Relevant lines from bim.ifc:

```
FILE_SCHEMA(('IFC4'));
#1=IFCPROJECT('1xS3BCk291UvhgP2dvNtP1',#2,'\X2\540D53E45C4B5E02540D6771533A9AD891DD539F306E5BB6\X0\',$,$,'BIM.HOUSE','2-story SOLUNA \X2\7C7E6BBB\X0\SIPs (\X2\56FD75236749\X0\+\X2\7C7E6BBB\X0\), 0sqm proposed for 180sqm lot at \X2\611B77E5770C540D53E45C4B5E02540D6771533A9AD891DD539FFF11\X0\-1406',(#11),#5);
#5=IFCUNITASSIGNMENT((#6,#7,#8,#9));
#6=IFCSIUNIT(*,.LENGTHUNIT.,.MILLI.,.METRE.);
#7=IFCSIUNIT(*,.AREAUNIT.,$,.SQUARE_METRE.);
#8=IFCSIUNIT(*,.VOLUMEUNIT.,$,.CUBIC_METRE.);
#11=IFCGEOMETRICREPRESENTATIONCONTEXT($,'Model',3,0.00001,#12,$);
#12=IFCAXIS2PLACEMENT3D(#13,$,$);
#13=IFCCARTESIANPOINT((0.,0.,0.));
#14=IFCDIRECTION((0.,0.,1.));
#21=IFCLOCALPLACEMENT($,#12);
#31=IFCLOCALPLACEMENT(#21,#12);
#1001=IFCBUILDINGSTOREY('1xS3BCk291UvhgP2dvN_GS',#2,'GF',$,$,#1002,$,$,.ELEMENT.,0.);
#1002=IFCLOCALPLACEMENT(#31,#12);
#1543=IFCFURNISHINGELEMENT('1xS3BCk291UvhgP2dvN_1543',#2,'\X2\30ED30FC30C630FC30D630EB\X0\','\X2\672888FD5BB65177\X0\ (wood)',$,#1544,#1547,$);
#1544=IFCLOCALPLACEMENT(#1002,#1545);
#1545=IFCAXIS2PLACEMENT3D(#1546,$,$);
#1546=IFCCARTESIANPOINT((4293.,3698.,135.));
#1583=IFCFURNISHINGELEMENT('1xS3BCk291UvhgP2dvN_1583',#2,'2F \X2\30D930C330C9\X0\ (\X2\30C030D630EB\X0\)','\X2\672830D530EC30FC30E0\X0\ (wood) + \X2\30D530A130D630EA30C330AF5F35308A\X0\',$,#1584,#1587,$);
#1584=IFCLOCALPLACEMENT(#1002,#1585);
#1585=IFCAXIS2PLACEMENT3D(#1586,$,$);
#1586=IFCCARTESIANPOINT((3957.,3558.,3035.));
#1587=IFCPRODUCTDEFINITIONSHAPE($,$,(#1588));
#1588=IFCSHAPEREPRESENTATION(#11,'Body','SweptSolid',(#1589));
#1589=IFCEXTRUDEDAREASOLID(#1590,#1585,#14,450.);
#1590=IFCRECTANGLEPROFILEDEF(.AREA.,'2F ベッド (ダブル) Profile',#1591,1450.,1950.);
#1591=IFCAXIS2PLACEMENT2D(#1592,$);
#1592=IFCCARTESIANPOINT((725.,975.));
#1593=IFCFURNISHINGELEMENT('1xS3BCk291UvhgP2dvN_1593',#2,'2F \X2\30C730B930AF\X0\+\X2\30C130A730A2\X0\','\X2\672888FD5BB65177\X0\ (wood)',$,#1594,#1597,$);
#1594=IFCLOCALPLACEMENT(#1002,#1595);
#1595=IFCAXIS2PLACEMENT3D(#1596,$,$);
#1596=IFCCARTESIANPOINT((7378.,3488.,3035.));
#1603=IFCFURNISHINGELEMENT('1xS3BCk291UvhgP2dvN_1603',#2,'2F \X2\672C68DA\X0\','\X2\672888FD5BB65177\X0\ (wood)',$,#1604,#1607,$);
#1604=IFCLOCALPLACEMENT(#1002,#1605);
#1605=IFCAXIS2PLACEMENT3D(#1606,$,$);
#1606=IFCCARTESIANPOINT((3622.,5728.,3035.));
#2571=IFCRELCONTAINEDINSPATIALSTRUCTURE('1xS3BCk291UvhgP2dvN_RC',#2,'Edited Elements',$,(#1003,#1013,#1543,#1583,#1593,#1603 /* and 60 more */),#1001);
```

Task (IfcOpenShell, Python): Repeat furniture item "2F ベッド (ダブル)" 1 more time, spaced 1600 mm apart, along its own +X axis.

```python
import ifcopenshell
import ifcopenshell.api.geometry
import ifcopenshell.api.root
import ifcopenshell.util.element
import ifcopenshell.util.placement

model = ifcopenshell.open("bim.ifc")


def reuse_history(source, copy):
    """copy_class also copies each property set's owner history, people and application; keep the originals."""
    for rel in copy.IsDefinedBy:
        if rel.is_a("IfcRelDefinesByProperties") and (history := rel.RelatingPropertyDefinition.OwnerHistory):
            rel.RelatingPropertyDefinition.OwnerHistory = source.OwnerHistory
            ifcopenshell.util.element.remove_deep2(model, history)


source = model.by_id(1583)
base = ifcopenshell.util.placement.get_local_placement(source.ObjectPlacement)
step = base[:3, 0] * 1600.0

for i in range(1, 2):
    copy = ifcopenshell.api.root.copy_class(model, product=source)
    copy.Representation = ifcopenshell.util.element.copy_deep(
        model, source.Representation, exclude=["IfcGeometricRepresentationContext", "IfcRepresentationMap"]
    )
    reuse_history(source, copy)
    matrix = base.copy()
    matrix[:3, 3] += i * step
    print("added at", matrix[:3, 3].round(3) + 0.0)
    ifcopenshell.api.geometry.edit_object_placement(model, product=copy, matrix=matrix, is_si=False)

model.write("bim_updated.ifc")
```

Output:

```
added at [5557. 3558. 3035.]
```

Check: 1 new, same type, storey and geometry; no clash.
